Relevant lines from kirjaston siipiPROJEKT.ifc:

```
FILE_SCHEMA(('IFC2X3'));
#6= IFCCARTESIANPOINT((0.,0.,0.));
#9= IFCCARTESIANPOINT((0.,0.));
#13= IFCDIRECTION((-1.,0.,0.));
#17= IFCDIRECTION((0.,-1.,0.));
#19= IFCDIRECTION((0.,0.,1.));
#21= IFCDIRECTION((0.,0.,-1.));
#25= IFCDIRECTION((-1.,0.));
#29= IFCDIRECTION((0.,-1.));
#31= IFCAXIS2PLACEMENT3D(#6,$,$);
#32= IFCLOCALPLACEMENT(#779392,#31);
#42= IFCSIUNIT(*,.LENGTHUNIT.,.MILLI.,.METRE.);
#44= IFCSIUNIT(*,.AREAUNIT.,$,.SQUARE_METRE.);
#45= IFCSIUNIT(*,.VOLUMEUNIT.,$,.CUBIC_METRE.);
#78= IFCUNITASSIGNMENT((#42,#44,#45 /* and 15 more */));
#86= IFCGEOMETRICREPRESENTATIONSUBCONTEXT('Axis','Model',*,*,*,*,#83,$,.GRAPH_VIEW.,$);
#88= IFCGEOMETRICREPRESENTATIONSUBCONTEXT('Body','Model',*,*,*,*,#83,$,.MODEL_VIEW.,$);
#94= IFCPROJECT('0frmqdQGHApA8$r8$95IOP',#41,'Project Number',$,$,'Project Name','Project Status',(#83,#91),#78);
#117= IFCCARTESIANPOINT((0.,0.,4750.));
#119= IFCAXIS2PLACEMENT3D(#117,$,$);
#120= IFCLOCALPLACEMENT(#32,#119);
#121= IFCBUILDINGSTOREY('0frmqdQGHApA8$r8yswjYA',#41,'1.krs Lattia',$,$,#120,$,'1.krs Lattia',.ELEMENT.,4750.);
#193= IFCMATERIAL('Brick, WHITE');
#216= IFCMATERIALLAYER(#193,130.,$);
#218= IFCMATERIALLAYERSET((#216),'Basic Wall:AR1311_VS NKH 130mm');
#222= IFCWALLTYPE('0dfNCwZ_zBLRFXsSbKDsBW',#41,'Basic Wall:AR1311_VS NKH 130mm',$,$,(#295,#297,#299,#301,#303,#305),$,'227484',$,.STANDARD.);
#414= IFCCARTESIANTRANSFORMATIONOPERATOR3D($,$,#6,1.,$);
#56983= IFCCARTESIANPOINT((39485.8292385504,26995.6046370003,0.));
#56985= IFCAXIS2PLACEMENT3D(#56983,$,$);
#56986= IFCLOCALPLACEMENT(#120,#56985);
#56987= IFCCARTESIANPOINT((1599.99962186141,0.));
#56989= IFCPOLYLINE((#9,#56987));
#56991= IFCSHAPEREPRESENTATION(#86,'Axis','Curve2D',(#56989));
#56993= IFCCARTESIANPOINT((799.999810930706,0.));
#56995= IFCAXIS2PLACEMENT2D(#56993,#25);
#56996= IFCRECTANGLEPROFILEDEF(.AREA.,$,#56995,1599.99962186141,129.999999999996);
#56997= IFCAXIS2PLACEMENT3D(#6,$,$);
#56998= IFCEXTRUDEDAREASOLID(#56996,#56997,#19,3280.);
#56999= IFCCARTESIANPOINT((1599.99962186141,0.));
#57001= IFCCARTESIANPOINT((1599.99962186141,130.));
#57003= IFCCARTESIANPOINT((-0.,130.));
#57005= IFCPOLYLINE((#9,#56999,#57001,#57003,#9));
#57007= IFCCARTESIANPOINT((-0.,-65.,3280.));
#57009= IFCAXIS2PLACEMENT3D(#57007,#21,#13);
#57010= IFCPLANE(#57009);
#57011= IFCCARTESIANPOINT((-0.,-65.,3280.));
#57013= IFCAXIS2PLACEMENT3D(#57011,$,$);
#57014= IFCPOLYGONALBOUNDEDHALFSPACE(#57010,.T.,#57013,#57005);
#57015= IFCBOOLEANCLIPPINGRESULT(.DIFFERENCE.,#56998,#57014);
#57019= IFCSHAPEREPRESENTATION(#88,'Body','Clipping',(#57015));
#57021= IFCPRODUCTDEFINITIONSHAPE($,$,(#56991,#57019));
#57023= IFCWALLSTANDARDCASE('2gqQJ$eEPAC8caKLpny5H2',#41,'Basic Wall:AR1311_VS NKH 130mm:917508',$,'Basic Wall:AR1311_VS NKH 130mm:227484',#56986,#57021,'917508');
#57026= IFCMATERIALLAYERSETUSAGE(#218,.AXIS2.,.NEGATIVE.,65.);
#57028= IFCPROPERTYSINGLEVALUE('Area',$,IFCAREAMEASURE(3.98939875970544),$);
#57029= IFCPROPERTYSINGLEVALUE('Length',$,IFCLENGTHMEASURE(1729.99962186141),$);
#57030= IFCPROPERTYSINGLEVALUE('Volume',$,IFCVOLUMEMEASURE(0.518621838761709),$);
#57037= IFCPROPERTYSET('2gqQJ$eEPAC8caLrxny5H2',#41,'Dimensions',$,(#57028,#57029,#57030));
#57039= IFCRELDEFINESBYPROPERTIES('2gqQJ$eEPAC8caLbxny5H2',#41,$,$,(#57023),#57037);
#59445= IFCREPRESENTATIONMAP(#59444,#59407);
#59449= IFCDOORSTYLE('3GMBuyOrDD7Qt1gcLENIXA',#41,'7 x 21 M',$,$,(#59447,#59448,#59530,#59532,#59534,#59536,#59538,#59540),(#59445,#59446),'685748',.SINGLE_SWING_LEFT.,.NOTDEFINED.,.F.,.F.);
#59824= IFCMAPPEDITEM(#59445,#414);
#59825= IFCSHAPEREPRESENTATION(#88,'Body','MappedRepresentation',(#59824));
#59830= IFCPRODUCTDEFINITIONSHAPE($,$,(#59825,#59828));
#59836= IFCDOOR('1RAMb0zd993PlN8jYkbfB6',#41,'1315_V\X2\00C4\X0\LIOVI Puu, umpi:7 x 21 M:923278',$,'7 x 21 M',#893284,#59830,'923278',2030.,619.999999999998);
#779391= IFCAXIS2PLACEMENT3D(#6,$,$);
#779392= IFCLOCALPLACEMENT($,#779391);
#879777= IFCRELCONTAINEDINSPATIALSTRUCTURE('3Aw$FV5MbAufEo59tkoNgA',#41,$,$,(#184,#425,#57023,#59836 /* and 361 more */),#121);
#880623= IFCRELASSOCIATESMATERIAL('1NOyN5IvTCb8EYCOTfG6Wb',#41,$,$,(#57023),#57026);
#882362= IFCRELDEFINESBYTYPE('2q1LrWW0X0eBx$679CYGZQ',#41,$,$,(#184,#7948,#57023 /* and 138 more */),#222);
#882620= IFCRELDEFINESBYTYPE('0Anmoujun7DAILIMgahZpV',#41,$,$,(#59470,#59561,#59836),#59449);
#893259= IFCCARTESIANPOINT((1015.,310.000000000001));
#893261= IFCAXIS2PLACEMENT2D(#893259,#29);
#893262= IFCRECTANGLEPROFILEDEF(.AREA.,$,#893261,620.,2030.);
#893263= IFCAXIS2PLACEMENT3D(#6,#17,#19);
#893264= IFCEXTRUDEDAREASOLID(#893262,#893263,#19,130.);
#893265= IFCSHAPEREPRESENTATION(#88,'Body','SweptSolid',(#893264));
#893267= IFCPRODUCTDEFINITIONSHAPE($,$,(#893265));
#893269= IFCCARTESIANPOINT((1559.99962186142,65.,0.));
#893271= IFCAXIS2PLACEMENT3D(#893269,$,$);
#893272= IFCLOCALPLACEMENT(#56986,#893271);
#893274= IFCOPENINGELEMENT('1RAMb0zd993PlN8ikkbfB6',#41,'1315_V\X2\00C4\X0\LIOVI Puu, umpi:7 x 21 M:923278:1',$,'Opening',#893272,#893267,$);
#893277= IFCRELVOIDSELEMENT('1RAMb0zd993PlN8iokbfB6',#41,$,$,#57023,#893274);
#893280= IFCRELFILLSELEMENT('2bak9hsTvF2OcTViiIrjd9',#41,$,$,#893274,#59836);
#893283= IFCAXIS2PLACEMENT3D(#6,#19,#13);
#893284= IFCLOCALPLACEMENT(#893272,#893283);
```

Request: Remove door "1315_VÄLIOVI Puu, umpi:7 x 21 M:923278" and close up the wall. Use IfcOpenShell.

```python
import ifcopenshell
import ifcopenshell.api.feature
import ifcopenshell.api.pset
import ifcopenshell.api.root
import ifcopenshell.geom
import ifcopenshell.util.element
import ifcopenshell.util.shape
import ifcopenshell.util.unit

model = ifcopenshell.open("kirjaston siipiPROJEKT.ifc")
area_scale = ifcopenshell.util.unit.calculate_unit_scale(model, "AREAUNIT")
volume_scale = ifcopenshell.util.unit.calculate_unit_scale(model, "VOLUMEUNIT")
settings = ifcopenshell.geom.settings()


def volume(element):
    """Net volume in cubic metres, openings subtracted."""
    shape = ifcopenshell.geom.create_shape(settings, element)
    return ifcopenshell.util.shape.get_volume(shape.geometry)


door = model.by_guid("1RAMb0zd993PlN8jYkbfB6")
opening = door.FillsVoids[0].RelatingOpeningElement
wall = opening.VoidsElements[0].RelatingBuildingElement
before = volume(wall)

ifcopenshell.api.root.remove_product(model, product=door)
ifcopenshell.api.feature.remove_feature(model, feature=opening)

after = volume(wall)
thickness = 0.13  # wall thickness in metres

# Update the wall's stored quantities.
pset = model.by_id(ifcopenshell.util.element.get_pset(wall, "Dimensions", should_inherit=False)["id"])
ifcopenshell.api.pset.edit_pset(model, pset=pset, properties={
    "Area": model.create_entity("IfcAreaMeasure", after / thickness / area_scale),
    "Volume": model.create_entity("IfcVolumeMeasure", after / volume_scale),
})

print(f"wall volume {before:.3f} -> {after:.3f} m3")

model.write("kirjaston siipiPROJEKT_rev.ifc")
```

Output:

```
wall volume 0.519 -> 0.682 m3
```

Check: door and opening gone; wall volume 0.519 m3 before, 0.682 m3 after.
